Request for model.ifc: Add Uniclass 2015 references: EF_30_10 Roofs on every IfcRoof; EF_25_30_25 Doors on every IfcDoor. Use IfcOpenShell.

First a look at what the model holds.

```python
import ifcopenshell

model = ifcopenshell.open("model.ifc")
print(model.schema)
print("classifications:", [c.Name for c in model.by_type("IfcClassification")])
for ifc_class in ("IfcDoor", "IfcRoof", "IfcStair", "IfcWall", "IfcWindow"):
    print(ifc_class, len(model.by_type(ifc_class)))
```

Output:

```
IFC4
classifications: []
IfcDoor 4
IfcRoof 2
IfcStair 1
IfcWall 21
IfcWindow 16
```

```python
import ifcopenshell
import ifcopenshell.api.classification

model = ifcopenshell.open("model.ifc")

system = ifcopenshell.api.classification.add_classification(model, classification="Uniclass 2015")

codes = {
    "IfcRoof": ("EF_30_10", "Roofs"),
    "IfcDoor": ("EF_25_30_25", "Doors"),
}
for ifc_class, (code, name) in codes.items():
    products = model.by_type(ifc_class)
    ifcopenshell.api.classification.add_reference(
        model, products=products, classification=system, identification=code, name=name
    )
    print(code, len(products))

model.write("model_updated.ifc")
```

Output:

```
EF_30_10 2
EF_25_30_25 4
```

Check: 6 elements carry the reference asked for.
